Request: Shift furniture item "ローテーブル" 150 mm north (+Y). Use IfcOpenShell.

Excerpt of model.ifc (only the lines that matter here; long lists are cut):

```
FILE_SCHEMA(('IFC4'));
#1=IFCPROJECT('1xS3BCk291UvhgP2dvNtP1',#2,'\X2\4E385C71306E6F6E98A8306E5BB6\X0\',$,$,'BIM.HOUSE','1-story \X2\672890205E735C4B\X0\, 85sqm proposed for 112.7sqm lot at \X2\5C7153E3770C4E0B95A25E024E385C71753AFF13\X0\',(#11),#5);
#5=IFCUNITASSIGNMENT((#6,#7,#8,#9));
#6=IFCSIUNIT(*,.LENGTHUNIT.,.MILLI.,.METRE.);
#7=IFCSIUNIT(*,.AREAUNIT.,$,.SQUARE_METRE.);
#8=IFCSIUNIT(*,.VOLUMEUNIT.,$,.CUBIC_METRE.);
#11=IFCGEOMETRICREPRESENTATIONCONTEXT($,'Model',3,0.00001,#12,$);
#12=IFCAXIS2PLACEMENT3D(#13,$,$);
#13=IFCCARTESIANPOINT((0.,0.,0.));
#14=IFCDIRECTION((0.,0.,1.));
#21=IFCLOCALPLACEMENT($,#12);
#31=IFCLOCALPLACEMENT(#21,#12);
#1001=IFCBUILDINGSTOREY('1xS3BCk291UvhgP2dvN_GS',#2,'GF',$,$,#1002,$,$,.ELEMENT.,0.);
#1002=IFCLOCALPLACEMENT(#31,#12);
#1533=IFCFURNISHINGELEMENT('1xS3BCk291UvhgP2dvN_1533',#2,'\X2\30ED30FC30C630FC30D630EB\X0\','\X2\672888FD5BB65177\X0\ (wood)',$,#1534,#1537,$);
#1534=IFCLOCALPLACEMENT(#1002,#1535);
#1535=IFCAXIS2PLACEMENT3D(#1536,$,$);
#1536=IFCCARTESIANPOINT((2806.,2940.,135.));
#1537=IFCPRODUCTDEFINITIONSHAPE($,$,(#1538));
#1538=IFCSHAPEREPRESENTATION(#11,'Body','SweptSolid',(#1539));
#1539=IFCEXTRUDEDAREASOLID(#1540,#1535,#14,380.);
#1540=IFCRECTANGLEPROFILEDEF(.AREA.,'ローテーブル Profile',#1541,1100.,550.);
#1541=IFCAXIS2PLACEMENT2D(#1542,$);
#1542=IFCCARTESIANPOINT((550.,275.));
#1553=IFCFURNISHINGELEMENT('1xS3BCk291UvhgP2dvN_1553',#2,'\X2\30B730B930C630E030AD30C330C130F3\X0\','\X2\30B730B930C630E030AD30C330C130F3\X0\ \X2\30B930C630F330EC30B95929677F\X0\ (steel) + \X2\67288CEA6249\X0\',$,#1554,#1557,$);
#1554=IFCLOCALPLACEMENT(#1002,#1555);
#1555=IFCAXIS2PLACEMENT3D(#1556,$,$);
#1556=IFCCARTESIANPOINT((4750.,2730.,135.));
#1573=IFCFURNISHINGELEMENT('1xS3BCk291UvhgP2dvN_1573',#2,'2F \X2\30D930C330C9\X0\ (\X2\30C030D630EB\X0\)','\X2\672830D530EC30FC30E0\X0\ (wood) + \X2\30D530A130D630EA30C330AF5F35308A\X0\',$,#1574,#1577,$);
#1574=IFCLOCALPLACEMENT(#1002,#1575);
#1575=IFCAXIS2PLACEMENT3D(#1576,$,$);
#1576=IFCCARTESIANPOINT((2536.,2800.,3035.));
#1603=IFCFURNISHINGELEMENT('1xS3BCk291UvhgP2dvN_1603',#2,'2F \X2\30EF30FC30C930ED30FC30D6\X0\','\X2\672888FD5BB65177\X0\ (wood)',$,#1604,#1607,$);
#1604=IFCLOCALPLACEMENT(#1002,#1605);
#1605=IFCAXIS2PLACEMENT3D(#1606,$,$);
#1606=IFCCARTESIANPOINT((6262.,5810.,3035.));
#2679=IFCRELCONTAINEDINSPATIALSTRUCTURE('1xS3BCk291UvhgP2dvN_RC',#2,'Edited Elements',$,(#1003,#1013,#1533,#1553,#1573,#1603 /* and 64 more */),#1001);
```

```python
import ifcopenshell
import ifcopenshell.api.geometry
import ifcopenshell.util.placement

model = ifcopenshell.open("model.ifc")

item = model.by_guid("1xS3BCk291UvhgP2dvN_1533")
matrix = ifcopenshell.util.placement.get_local_placement(item.ObjectPlacement)
matrix[1, 3] += 150.0
ifcopenshell.api.geometry.edit_object_placement(model, product=item, matrix=matrix, is_si=False)

print(ifcopenshell.util.placement.get_local_placement(item.ObjectPlacement).round(3) + 0.0)

model.write("model_updated.ifc")
```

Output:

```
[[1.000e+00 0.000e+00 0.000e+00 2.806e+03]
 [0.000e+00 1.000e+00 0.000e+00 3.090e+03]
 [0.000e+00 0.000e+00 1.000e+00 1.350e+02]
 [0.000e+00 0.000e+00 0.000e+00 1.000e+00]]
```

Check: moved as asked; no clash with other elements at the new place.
